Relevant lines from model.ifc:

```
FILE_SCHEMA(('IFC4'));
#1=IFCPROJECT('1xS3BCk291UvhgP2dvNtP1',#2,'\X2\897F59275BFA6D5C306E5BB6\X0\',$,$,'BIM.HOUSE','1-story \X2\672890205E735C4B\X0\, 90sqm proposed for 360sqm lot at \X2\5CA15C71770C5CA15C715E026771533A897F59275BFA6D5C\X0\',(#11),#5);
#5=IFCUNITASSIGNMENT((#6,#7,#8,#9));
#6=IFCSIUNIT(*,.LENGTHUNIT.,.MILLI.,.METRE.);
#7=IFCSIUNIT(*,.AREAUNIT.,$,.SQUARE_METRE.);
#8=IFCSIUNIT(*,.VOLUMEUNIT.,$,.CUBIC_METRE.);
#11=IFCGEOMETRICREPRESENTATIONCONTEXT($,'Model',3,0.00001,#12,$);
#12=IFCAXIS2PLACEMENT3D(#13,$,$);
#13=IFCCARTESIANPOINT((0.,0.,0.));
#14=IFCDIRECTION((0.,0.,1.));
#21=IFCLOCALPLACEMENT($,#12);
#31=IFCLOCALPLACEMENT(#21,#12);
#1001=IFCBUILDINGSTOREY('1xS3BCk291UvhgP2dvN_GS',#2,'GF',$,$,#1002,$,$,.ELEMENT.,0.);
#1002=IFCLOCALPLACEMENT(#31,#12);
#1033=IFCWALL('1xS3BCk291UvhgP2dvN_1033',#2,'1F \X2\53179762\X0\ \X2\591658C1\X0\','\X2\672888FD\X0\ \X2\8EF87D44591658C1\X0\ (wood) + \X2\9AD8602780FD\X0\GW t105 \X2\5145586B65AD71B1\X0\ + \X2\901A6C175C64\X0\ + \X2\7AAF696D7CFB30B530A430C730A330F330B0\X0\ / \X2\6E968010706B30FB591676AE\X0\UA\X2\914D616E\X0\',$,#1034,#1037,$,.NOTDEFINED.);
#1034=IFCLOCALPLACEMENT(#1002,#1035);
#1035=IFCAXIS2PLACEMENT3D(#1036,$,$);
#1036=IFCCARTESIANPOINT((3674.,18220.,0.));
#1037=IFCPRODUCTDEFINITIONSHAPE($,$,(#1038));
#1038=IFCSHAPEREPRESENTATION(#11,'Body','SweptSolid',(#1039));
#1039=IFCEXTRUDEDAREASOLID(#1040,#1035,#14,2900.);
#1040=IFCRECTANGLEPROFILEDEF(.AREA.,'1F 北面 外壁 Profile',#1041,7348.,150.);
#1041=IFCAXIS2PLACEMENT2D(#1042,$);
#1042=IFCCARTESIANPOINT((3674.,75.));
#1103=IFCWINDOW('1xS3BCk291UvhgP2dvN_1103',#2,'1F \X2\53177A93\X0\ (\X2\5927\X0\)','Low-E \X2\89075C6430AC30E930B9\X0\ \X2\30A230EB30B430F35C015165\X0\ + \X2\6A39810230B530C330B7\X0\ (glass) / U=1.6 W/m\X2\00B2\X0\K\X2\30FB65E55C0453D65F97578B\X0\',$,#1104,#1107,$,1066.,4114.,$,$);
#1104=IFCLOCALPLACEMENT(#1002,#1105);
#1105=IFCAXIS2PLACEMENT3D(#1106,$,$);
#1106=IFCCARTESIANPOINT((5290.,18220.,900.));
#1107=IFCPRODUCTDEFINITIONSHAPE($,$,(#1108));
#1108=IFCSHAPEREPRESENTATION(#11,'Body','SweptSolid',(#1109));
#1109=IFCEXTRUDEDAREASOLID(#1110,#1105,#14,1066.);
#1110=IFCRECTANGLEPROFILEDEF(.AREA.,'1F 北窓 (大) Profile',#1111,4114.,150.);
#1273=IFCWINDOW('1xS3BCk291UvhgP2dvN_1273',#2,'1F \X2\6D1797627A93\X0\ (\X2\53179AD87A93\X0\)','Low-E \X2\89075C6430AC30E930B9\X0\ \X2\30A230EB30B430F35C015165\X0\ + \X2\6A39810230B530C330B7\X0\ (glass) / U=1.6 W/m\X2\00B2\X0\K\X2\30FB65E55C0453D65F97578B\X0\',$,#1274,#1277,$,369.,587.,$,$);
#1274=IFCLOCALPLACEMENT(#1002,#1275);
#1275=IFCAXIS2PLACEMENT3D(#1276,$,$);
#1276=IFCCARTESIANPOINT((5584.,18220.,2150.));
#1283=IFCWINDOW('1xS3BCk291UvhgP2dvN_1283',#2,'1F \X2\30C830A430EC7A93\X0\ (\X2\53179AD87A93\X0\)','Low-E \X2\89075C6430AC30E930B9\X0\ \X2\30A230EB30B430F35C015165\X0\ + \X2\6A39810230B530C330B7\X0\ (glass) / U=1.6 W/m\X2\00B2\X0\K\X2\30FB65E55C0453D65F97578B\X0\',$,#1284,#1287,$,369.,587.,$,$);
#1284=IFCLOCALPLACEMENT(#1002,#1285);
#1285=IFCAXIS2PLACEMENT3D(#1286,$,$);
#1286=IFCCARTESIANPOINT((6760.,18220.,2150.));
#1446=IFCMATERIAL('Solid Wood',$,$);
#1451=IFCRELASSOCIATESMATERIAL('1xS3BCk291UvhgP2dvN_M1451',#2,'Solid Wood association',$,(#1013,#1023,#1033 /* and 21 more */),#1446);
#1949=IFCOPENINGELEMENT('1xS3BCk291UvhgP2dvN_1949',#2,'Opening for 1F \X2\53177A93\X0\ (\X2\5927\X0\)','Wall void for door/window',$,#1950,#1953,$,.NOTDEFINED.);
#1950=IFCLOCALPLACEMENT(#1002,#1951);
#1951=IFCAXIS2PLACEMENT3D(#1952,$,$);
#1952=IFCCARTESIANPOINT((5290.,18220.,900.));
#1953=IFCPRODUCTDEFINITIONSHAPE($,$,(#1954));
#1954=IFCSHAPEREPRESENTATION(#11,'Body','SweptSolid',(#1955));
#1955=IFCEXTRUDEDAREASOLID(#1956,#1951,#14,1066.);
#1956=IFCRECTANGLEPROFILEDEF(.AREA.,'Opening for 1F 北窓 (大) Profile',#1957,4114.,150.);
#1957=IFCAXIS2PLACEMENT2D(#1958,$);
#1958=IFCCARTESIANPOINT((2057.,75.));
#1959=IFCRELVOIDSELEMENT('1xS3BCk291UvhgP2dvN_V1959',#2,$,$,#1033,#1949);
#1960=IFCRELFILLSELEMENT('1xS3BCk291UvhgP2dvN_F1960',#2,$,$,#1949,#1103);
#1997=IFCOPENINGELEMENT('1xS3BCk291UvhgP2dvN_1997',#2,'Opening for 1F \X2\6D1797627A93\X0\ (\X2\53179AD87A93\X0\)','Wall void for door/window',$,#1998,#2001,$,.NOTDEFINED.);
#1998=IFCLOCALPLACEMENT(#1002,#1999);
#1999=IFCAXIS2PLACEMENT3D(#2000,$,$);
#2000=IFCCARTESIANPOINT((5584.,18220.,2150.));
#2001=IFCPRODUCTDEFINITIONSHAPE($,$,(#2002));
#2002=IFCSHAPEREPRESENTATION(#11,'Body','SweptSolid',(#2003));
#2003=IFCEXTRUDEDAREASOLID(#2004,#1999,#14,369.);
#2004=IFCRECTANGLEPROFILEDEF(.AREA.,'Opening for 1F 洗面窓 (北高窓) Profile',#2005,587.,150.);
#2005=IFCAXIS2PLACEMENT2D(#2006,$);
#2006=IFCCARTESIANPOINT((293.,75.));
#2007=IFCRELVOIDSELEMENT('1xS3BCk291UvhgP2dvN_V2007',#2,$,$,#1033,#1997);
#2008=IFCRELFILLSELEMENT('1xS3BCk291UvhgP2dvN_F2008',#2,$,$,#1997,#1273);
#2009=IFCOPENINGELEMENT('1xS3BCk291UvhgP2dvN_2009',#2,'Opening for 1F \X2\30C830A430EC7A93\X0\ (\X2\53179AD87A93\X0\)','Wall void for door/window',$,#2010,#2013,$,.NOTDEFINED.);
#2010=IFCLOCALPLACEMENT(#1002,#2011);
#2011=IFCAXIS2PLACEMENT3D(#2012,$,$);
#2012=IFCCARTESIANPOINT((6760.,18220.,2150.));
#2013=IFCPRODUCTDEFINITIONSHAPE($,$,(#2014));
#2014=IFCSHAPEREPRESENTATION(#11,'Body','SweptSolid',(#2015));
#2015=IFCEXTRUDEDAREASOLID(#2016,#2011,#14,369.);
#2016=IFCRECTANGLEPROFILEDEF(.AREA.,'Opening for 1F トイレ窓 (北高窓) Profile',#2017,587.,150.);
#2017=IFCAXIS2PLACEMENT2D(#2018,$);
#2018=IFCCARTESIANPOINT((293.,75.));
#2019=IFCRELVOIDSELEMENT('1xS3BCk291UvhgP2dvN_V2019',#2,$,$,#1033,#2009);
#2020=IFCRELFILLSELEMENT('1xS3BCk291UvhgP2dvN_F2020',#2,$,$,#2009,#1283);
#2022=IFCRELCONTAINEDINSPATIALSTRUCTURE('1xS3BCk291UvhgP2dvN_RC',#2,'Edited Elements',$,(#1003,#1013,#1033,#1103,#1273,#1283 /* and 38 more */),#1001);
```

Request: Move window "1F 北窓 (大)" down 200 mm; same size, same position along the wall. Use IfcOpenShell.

```python
import numpy as np
import ifcopenshell
import ifcopenshell.api.geometry
import ifcopenshell.util.placement
import ifcopenshell.util.unit

model = ifcopenshell.open("model.ifc")
unit_scale = ifcopenshell.util.unit.calculate_unit_scale(model)

window = model.by_id(1103)
opening = window.FillsVoids[0].RelatingOpeningElement
dz = -200.0

shift = np.array([0.0, 0.0, dz])
# The window is not placed relative to its opening, so move both.
for product in (opening, window):
    matrix = ifcopenshell.util.placement.get_local_placement(product.ObjectPlacement)
    matrix[:3, 3] += shift
    ifcopenshell.api.geometry.edit_object_placement(model, product=product, matrix=matrix, is_si=False)

print(f"moved by {dz * unit_scale:+.3f} m")

model.write("model_rev.ifc")
```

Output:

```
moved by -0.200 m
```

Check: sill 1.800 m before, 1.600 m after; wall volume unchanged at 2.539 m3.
